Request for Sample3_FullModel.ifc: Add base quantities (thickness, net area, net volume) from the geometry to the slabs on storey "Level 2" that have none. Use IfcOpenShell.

First a look at what the model holds.

```python
import ifcopenshell
import ifcopenshell.util.element
import ifcopenshell.util.unit

model = ifcopenshell.open("Sample3_FullModel.ifc")
print(model.schema)
for unit_type in ("LENGTHUNIT", "AREAUNIT", "VOLUMEUNIT"):
    print(unit_type, ifcopenshell.util.unit.calculate_unit_scale(model, unit_type))
storey = next(s for s in model.by_type("IfcBuildingStorey") if s.Name == "Level 2")
slabs = [e for e in ifcopenshell.util.element.get_decomposition(storey) if e.is_a("IfcSlab")]
for e in sorted(slabs, key=lambda e: e.id()):
    print(e.id(), e.is_a(), e.Name, list(ifcopenshell.util.element.get_psets(e, qtos_only=True)), sep=" | ")
```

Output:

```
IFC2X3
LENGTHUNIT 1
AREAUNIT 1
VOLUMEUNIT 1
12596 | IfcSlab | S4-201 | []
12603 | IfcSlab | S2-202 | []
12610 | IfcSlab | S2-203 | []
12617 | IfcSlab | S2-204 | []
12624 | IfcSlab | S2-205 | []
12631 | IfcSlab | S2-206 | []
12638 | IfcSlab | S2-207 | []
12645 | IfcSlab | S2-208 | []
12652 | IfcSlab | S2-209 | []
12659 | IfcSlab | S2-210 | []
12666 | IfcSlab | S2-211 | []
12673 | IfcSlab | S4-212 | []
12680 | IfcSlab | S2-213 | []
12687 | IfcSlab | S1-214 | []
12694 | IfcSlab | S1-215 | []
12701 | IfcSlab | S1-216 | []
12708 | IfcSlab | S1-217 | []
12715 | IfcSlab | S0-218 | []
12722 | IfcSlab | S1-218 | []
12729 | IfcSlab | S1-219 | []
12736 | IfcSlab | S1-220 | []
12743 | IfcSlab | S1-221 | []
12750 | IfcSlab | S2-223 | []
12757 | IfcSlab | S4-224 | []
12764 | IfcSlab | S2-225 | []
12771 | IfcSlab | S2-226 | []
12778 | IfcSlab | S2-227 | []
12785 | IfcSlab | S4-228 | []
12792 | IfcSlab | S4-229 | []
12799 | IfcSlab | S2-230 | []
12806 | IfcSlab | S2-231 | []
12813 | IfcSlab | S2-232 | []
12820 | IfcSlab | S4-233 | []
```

```python
import ifcopenshell
import ifcopenshell.api.pset
import ifcopenshell.geom
import ifcopenshell.util.element
import ifcopenshell.util.shape
import ifcopenshell.util.unit

model = ifcopenshell.open("Sample3_FullModel.ifc")
unit_scale = ifcopenshell.util.unit.calculate_unit_scale(model)
area_scale = ifcopenshell.util.unit.calculate_unit_scale(model, "AREAUNIT")
volume_scale = ifcopenshell.util.unit.calculate_unit_scale(model, "VOLUMEUNIT")
settings = ifcopenshell.geom.settings()

storey = next(s for s in model.by_type("IfcBuildingStorey") if s.Name == "Level 2")
slabs = [e for e in ifcopenshell.util.element.get_decomposition(storey) if e.is_a("IfcSlab")]

for e in sorted(slabs, key=lambda e: e.id()):
    if ifcopenshell.util.element.get_psets(e, qtos_only=True, should_inherit=False):
        continue
    # Geometry comes back in metres, in the element's own axes.
    shape = ifcopenshell.geom.create_shape(settings, e)
    values = {
        "Width": ifcopenshell.util.shape.get_z(shape.geometry) / unit_scale,
        "NetArea": ifcopenshell.util.shape.get_footprint_area(shape.geometry) / area_scale,
        "NetVolume": ifcopenshell.util.shape.get_volume(shape.geometry) / volume_scale,
    }
    qto = ifcopenshell.api.pset.add_qto(model, product=e, name="BaseQuantities")
    ifcopenshell.api.pset.edit_qto(model, qto=qto, properties=values)
    print(e.id(), {k: round(v, 3) for k, v in values.items()})

model.write("Sample3_FullModel_updated.ifc")
```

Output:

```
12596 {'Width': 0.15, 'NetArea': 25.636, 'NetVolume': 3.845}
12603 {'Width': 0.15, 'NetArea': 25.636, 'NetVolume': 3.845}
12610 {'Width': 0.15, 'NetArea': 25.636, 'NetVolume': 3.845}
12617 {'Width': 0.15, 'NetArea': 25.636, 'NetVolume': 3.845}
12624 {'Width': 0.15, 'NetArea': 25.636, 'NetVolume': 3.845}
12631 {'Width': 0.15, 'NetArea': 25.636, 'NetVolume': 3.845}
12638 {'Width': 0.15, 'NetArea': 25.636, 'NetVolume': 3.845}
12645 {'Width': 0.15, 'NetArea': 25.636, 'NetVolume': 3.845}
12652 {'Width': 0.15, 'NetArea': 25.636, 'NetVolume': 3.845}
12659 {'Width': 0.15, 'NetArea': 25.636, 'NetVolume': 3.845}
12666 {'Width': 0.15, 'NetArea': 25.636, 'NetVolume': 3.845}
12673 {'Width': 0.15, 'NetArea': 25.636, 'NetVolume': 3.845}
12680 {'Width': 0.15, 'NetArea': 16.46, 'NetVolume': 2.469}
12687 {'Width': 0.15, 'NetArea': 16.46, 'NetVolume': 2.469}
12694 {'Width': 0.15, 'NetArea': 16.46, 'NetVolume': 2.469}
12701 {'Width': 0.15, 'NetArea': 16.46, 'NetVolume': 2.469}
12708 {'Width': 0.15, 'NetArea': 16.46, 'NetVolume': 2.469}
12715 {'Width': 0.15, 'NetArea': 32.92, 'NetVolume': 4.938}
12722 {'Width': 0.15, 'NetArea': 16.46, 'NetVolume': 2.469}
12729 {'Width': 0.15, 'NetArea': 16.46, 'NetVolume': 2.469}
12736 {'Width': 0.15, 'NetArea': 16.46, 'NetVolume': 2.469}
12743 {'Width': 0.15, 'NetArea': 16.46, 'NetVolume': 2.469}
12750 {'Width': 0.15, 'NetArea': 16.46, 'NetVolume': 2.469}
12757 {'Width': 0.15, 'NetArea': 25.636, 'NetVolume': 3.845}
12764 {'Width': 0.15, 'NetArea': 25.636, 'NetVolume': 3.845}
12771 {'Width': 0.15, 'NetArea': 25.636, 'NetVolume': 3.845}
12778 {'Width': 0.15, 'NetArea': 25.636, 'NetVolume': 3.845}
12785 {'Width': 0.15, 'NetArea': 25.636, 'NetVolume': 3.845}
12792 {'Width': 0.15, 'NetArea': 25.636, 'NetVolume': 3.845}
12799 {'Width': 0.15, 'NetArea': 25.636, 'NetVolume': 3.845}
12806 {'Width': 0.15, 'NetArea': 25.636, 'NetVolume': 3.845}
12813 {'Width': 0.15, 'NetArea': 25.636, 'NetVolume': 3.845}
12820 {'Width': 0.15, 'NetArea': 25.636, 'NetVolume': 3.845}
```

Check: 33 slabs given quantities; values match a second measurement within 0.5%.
